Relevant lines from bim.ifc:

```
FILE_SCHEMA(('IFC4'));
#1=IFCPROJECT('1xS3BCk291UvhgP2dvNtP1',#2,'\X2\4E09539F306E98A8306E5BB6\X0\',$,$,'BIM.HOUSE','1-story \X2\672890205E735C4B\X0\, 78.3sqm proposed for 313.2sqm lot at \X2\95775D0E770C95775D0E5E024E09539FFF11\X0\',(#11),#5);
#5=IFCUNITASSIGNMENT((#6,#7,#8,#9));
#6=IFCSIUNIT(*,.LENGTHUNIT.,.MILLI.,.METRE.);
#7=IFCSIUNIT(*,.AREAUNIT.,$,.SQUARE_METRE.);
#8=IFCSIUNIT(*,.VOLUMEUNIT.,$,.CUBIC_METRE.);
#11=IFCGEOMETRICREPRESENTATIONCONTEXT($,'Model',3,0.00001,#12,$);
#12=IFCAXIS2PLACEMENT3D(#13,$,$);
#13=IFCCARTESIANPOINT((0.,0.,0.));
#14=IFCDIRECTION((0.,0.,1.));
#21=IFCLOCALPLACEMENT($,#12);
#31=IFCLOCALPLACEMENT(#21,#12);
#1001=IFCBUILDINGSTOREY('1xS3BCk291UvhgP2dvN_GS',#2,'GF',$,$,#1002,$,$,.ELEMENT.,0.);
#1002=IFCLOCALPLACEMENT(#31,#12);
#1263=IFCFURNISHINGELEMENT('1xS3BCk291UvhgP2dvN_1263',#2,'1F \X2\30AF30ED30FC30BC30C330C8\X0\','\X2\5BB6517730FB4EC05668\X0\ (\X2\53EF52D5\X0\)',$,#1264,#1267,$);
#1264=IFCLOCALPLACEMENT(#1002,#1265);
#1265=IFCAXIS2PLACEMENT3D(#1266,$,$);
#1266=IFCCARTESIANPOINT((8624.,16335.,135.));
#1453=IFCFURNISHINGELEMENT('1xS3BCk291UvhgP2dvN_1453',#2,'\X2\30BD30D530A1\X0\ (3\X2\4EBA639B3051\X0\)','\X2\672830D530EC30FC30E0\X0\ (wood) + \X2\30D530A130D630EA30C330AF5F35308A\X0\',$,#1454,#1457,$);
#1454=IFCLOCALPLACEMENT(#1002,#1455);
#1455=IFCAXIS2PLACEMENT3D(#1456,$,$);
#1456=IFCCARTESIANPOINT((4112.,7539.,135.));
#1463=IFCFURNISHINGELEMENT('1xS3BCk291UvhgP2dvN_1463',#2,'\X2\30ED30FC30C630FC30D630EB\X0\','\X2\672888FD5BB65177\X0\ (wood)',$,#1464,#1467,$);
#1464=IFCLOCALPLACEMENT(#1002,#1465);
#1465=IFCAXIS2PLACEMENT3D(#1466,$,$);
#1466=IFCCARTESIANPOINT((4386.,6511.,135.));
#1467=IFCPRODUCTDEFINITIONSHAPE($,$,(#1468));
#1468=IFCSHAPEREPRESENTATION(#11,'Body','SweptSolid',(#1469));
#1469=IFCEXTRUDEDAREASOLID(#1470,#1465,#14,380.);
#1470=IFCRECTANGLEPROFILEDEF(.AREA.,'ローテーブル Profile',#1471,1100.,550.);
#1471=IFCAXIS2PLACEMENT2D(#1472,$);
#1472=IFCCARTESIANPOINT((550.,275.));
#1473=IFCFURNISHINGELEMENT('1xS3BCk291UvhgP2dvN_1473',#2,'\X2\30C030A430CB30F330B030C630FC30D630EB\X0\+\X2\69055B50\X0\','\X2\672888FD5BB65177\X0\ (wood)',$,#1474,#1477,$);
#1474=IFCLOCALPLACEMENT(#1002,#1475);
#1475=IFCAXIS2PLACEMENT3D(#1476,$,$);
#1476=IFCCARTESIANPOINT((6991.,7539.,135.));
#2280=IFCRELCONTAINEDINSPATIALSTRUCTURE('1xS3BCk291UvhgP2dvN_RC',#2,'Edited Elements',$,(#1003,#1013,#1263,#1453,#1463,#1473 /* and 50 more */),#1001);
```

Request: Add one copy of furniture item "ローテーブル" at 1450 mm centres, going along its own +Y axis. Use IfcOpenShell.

```python
import ifcopenshell
import ifcopenshell.api.geometry
import ifcopenshell.api.root
import ifcopenshell.util.element
import ifcopenshell.util.placement
import ifcopenshell.util.unit

model = ifcopenshell.open("bim.ifc")
unit_scale = ifcopenshell.util.unit.calculate_unit_scale(model)


def reuse_history(source, copy):
    """copy_class also copies each property set's owner history, people and application; keep the originals."""
    for rel in copy.IsDefinedBy:
        if rel.is_a("IfcRelDefinesByProperties") and (history := rel.RelatingPropertyDefinition.OwnerHistory):
            rel.RelatingPropertyDefinition.OwnerHistory = source.OwnerHistory
            ifcopenshell.util.element.remove_deep2(model, history)


source = model.by_guid("1xS3BCk291UvhgP2dvN_1463")
base = ifcopenshell.util.placement.get_local_placement(source.ObjectPlacement)
step = base[:3, 1] * 1.45 / unit_scale

for i in range(1, 2):
    copy = ifcopenshell.api.root.copy_class(model, product=source)
    copy.Representation = ifcopenshell.util.element.copy_deep(
        model, source.Representation, exclude=["IfcGeometricRepresentationContext", "IfcRepresentationMap"]
    )
    reuse_history(source, copy)
    matrix = base.copy()
    matrix[:3, 3] += i * step
    print("added at", matrix[:3, 3].round(3) + 0.0)
    ifcopenshell.api.geometry.edit_object_placement(model, product=copy, matrix=matrix, is_si=False)

model.write("bim_rev.ifc")
```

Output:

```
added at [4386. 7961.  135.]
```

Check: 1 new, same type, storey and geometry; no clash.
